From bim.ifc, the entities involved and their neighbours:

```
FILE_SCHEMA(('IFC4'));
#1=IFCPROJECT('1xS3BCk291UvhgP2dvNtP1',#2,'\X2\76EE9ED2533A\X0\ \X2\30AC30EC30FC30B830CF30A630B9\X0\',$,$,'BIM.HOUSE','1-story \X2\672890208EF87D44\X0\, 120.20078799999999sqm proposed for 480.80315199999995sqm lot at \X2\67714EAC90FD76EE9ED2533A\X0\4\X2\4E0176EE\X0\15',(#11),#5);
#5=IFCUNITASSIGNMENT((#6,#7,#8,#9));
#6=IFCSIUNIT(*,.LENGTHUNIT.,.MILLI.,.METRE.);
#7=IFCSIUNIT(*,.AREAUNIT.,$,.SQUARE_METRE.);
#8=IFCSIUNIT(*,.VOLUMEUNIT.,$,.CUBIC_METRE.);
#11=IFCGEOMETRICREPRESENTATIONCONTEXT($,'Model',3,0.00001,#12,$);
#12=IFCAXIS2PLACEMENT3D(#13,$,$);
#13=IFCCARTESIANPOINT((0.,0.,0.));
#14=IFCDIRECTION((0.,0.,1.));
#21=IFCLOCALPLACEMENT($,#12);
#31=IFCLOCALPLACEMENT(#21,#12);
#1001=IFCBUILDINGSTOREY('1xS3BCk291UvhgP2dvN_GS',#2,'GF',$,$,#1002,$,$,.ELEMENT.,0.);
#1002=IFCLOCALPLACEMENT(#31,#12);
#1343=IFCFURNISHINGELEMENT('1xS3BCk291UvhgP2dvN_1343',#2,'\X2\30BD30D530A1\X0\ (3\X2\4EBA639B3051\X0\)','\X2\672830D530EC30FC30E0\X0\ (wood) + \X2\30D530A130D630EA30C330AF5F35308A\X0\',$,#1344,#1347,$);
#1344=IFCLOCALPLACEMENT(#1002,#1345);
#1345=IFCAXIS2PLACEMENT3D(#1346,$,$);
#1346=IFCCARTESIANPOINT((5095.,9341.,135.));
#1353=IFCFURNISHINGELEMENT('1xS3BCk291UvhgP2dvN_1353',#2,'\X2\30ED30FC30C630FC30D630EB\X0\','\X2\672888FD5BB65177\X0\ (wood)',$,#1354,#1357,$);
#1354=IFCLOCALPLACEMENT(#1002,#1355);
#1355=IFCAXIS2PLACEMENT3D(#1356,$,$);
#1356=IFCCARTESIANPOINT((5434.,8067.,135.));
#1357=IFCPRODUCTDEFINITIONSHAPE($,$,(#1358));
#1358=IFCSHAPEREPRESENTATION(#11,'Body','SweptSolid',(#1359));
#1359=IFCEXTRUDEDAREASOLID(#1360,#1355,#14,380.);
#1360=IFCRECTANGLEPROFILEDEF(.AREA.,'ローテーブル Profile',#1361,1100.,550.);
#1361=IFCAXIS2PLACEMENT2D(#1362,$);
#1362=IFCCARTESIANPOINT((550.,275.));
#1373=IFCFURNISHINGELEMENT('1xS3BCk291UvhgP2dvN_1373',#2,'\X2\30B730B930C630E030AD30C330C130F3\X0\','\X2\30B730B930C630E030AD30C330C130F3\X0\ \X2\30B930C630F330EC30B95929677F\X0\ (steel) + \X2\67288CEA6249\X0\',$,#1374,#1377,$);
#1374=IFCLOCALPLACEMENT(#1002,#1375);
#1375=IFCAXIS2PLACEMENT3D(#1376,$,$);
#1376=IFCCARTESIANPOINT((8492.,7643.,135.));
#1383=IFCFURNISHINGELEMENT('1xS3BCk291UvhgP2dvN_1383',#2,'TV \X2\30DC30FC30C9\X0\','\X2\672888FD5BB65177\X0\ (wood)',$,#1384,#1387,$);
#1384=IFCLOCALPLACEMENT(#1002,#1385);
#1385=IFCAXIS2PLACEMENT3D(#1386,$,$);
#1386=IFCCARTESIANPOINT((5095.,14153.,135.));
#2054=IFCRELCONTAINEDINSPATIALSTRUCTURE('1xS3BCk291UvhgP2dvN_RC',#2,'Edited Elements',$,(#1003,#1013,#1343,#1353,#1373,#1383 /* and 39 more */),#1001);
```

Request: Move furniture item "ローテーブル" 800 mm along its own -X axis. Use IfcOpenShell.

```python
import ifcopenshell
import ifcopenshell.api.geometry
import ifcopenshell.util.placement
import ifcopenshell.util.unit

model = ifcopenshell.open("bim.ifc")
unit_scale = ifcopenshell.util.unit.calculate_unit_scale(model)

item = model.by_guid("1xS3BCk291UvhgP2dvN_1353")
matrix = ifcopenshell.util.placement.get_local_placement(item.ObjectPlacement)
matrix[:3, 3] -= matrix[:3, 0] * 0.8 / unit_scale
ifcopenshell.api.geometry.edit_object_placement(model, product=item, matrix=matrix, is_si=False)

print(ifcopenshell.util.placement.get_local_placement(item.ObjectPlacement).round(3) + 0.0)

model.write("bim_v2.ifc")
```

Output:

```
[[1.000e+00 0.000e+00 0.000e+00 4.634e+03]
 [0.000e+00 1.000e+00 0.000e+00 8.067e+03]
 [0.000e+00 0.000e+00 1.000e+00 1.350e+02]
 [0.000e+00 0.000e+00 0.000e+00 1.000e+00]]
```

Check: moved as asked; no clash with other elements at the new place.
